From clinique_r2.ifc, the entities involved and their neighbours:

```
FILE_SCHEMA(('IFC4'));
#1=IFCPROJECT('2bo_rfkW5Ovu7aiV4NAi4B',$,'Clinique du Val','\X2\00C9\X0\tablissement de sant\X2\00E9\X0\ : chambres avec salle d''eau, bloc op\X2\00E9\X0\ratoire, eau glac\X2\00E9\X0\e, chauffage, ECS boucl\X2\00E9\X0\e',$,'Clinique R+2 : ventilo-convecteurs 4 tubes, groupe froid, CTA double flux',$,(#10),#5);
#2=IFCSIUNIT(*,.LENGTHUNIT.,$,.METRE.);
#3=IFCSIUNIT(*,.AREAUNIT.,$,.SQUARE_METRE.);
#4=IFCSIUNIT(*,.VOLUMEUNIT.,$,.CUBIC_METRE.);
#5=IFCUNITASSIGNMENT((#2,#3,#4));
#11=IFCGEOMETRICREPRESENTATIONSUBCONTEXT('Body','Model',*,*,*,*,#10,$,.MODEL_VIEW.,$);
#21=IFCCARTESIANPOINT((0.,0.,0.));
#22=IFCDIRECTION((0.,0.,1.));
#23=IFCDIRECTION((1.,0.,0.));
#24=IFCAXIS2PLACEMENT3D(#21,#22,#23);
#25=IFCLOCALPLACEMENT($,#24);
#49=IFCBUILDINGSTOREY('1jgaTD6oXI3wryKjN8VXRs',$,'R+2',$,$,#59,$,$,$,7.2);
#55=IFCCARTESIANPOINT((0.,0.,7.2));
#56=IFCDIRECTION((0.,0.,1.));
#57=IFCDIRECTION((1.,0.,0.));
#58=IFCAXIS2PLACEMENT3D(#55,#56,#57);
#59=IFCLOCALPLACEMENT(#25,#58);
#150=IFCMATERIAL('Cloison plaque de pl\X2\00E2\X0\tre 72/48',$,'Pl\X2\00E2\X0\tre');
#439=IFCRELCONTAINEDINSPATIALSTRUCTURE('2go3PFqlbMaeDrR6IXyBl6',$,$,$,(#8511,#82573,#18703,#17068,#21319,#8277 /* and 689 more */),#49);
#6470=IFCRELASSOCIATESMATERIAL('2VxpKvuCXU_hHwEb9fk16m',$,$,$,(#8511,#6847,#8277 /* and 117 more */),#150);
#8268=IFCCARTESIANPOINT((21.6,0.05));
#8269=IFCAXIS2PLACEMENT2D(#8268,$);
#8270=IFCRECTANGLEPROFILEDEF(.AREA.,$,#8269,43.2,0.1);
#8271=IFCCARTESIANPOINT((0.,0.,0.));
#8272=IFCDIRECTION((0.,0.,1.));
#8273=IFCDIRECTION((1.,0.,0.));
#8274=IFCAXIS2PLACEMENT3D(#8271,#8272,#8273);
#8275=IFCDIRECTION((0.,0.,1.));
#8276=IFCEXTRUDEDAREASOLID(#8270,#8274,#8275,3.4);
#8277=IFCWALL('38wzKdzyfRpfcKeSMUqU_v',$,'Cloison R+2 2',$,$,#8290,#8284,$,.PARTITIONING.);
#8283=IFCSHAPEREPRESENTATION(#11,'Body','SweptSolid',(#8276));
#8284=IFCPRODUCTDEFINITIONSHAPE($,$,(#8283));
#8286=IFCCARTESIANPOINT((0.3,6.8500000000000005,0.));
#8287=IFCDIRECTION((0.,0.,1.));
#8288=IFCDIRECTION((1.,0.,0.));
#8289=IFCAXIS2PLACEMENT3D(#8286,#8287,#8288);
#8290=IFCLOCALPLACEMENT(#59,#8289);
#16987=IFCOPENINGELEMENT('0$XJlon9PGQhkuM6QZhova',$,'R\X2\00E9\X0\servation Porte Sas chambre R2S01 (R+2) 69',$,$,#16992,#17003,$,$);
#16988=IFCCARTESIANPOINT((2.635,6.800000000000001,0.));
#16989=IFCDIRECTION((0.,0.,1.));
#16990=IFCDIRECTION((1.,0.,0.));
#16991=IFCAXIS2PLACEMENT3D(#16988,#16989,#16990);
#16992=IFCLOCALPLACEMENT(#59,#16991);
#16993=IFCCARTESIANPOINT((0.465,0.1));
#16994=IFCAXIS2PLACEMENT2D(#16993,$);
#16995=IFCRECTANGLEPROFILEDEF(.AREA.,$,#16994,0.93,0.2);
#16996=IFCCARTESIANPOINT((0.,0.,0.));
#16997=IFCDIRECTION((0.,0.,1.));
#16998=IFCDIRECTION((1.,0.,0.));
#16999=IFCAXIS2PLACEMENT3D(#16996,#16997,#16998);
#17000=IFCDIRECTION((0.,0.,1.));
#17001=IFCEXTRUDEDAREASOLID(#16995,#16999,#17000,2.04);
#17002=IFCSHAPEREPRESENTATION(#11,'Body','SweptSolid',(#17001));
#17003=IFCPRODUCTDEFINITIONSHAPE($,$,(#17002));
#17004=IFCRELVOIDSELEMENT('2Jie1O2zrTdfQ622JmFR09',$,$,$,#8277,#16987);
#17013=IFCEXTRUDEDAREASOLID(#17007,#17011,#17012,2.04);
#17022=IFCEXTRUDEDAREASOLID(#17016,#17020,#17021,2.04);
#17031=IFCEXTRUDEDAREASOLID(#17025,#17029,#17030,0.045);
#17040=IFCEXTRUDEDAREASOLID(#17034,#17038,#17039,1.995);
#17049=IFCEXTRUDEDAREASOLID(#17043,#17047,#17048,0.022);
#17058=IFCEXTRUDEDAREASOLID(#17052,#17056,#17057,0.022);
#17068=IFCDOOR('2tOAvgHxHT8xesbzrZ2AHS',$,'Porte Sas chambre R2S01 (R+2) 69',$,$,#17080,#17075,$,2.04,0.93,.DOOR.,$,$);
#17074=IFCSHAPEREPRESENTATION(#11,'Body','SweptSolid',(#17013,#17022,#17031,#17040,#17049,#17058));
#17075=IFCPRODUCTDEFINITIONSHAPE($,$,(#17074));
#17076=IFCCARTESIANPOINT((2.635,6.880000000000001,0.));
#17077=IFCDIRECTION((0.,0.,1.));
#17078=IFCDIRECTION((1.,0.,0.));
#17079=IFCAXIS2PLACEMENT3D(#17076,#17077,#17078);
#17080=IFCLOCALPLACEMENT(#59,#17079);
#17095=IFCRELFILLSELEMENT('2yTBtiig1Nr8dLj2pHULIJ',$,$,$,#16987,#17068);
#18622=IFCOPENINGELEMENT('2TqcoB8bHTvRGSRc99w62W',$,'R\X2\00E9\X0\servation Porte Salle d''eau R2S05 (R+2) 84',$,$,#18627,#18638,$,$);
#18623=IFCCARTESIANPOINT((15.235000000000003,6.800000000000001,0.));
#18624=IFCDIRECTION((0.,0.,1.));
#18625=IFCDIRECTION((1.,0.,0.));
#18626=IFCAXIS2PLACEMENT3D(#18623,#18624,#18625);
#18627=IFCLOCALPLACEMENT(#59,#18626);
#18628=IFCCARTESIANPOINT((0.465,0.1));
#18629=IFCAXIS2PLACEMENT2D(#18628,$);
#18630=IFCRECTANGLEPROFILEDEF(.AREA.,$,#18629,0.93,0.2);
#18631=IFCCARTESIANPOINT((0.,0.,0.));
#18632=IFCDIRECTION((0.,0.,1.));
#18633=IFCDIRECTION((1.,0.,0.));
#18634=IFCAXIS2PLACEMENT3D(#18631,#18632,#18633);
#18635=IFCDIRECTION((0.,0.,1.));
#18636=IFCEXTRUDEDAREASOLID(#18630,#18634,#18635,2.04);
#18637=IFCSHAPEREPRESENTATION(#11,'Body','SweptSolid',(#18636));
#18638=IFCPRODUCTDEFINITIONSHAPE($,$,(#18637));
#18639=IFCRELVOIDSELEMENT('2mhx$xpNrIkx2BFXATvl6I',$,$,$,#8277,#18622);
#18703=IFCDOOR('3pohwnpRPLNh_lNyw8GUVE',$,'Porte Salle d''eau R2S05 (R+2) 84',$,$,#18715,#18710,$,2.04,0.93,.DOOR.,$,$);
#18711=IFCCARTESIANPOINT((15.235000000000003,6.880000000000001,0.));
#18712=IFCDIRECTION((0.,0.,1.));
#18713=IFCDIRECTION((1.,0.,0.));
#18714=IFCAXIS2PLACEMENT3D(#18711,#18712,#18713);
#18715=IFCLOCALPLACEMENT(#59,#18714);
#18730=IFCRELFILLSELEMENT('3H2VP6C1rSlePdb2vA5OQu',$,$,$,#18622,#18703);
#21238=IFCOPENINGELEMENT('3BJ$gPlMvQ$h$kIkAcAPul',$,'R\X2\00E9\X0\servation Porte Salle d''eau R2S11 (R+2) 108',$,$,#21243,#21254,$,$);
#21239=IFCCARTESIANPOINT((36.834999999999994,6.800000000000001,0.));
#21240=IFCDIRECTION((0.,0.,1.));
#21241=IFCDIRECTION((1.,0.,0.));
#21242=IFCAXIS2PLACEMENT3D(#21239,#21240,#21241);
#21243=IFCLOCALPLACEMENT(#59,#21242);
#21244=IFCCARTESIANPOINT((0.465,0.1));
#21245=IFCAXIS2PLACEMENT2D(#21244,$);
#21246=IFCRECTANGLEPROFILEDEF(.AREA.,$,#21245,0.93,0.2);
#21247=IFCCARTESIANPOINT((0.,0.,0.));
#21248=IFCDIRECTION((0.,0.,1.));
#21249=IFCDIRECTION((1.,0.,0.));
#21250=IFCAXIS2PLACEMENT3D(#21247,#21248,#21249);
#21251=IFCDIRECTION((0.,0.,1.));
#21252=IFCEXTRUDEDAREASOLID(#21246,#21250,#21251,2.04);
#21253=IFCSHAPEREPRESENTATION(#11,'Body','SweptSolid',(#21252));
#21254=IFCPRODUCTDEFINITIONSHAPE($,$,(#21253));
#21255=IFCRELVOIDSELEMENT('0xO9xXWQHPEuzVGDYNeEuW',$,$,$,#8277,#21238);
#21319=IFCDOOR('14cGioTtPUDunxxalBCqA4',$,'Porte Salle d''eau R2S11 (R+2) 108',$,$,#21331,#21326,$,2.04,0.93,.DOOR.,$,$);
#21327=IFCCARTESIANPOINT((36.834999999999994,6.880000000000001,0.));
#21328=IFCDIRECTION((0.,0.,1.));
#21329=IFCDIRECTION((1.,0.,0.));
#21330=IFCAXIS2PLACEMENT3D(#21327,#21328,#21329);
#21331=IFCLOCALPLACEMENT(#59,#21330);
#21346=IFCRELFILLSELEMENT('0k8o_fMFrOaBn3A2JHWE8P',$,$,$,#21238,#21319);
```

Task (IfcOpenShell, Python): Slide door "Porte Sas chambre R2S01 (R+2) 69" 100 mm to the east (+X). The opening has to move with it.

```python
import ifcopenshell
import ifcopenshell.api.geometry
import ifcopenshell.util.placement
import ifcopenshell.util.unit

model = ifcopenshell.open("clinique_r2.ifc")
unit_scale = ifcopenshell.util.unit.calculate_unit_scale(model)

door = model.by_guid("2tOAvgHxHT8xesbzrZ2AHS")
opening = door.FillsVoids[0].RelatingOpeningElement
wall = opening.VoidsElements[0].RelatingBuildingElement

wall_matrix = ifcopenshell.util.placement.get_local_placement(wall.ObjectPlacement)
shift = wall_matrix[:3, 0] * 0.1 / unit_scale
before = ifcopenshell.util.placement.get_local_placement(door.ObjectPlacement)[:3, 3].copy()

# The door is not placed relative to its opening, so move both.
for product in (opening, door):
    matrix = ifcopenshell.util.placement.get_local_placement(product.ObjectPlacement)
    matrix[:3, 3] += shift
    ifcopenshell.api.geometry.edit_object_placement(model, product=product, matrix=matrix, is_si=False)

after = ifcopenshell.util.placement.get_local_placement(door.ObjectPlacement)[:3, 3]
print("door moved by", (after - before).round(3) + 0.0)

model.write("clinique_r2_updated.ifc")
```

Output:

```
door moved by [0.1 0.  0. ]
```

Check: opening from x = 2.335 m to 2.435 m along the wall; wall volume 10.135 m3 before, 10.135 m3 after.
